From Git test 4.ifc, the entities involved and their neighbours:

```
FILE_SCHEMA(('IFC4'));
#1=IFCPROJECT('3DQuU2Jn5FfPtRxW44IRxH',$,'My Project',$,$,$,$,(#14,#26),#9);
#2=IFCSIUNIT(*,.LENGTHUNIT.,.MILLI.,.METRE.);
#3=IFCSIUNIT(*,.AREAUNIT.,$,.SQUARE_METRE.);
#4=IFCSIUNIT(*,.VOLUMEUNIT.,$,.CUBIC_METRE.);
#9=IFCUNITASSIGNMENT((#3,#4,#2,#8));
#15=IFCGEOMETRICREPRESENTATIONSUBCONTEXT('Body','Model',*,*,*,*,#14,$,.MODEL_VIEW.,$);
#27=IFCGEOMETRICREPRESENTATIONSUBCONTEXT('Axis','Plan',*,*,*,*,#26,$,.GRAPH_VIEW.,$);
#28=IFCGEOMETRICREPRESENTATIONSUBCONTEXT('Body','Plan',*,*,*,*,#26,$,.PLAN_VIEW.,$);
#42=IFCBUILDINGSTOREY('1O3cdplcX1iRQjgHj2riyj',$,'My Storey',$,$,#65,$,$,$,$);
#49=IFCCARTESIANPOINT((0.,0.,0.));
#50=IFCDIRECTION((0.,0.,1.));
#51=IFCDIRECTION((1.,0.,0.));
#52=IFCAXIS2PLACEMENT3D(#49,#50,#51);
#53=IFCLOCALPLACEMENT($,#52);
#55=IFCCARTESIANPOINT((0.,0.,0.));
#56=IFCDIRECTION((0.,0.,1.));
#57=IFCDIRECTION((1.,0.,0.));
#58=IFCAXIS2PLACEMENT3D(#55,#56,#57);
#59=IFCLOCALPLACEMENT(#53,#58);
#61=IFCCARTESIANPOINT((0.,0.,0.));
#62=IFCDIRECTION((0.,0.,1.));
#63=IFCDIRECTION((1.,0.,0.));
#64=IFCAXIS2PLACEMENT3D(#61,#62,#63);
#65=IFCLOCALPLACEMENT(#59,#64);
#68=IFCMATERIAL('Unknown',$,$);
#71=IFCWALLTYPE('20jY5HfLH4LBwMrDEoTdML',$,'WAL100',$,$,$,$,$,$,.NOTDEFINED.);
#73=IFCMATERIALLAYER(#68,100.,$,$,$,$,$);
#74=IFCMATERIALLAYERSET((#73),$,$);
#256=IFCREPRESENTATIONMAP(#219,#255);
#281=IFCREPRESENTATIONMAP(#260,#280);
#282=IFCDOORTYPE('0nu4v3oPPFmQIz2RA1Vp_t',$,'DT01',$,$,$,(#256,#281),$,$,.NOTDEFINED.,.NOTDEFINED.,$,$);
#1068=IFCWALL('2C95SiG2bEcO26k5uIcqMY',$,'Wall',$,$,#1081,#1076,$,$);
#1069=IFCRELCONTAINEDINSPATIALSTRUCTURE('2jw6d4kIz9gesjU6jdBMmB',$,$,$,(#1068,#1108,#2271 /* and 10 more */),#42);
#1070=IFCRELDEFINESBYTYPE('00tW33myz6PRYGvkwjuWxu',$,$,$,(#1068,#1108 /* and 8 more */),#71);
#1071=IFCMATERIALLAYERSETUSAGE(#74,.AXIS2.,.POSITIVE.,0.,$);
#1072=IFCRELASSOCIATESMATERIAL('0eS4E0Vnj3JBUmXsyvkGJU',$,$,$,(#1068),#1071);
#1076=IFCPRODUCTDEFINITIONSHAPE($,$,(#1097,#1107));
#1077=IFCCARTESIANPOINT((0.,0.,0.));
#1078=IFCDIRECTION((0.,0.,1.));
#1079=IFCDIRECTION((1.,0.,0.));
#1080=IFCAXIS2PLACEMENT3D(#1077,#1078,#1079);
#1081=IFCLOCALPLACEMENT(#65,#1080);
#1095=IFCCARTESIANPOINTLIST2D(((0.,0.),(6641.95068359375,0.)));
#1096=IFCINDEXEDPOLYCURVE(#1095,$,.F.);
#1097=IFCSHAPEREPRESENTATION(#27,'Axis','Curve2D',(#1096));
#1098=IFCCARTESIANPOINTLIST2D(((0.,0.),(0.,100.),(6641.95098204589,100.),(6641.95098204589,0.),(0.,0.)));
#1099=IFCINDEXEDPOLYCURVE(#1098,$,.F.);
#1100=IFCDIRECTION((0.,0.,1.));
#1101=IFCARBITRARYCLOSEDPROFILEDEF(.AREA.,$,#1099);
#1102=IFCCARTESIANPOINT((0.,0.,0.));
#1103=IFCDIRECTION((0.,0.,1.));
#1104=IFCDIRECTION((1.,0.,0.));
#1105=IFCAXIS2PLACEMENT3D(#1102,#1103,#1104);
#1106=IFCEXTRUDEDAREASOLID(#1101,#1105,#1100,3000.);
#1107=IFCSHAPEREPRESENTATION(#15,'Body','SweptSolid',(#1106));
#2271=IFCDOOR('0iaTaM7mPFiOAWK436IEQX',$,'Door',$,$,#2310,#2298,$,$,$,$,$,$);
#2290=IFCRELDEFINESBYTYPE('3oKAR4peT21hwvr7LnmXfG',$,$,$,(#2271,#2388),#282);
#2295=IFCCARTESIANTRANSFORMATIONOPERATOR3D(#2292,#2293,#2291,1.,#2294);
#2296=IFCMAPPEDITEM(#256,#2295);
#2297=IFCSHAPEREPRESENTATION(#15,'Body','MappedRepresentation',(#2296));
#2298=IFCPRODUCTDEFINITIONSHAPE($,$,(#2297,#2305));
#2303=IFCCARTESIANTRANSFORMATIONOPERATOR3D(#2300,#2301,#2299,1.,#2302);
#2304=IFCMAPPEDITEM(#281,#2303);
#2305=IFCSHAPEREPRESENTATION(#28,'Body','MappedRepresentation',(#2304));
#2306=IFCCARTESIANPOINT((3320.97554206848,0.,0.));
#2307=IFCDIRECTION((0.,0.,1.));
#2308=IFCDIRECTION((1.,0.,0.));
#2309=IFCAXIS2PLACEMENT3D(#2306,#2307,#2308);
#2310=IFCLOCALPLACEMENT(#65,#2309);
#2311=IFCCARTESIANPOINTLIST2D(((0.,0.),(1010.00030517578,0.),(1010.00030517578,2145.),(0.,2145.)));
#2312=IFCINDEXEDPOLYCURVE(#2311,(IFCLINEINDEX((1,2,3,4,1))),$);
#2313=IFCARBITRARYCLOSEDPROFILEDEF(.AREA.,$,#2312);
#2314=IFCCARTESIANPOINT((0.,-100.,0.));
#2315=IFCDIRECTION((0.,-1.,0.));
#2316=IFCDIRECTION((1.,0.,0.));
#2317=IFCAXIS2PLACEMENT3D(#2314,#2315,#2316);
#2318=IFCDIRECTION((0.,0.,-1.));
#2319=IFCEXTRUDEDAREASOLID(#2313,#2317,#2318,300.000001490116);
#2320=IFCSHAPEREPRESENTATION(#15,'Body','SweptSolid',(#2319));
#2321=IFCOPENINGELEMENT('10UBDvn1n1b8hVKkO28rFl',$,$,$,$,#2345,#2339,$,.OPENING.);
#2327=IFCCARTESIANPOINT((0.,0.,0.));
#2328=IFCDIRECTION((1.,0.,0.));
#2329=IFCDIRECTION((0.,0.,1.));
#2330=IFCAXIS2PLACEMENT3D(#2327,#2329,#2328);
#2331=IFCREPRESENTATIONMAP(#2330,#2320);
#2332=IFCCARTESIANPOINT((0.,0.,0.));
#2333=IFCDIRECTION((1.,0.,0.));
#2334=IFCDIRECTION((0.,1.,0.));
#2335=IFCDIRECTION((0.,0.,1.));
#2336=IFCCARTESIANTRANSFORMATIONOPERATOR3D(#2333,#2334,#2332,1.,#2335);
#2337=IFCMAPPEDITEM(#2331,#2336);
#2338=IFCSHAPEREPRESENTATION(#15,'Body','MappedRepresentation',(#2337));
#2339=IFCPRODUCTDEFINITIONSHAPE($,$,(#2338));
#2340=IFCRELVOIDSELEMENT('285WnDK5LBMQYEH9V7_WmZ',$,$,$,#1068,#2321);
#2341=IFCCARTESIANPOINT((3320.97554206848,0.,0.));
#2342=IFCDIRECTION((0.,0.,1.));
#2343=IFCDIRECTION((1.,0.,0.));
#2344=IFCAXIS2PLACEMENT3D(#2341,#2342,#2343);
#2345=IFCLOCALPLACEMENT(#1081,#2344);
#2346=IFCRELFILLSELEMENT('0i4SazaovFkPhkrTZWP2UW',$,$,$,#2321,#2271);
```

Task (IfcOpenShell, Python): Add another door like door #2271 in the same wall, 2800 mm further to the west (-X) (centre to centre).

```python
import ifcopenshell
import ifcopenshell.api.feature
import ifcopenshell.api.geometry
import ifcopenshell.api.root
import ifcopenshell.geom
import ifcopenshell.util.element
import ifcopenshell.util.placement
import ifcopenshell.util.shape
import ifcopenshell.util.unit

model = ifcopenshell.open("Git test 4.ifc")
unit_scale = ifcopenshell.util.unit.calculate_unit_scale(model)
settings = ifcopenshell.geom.settings()


def volume(element):
    """Net volume in cubic metres, openings subtracted."""
    shape = ifcopenshell.geom.create_shape(settings, element)
    return ifcopenshell.util.shape.get_volume(shape.geometry)


door = model.by_guid("0iaTaM7mPFiOAWK436IEQX")
opening = door.FillsVoids[0].RelatingOpeningElement
wall = opening.VoidsElements[0].RelatingBuildingElement
before = volume(wall)
shift = ifcopenshell.util.placement.get_local_placement(wall.ObjectPlacement)[:3, 0] * -2.8 / unit_scale

# copy_class copies the void relationship, type, container and properties, but no geometry.
new_opening = ifcopenshell.api.root.copy_class(model, product=opening)
new_opening.Representation = ifcopenshell.util.element.copy_deep(
    model, opening.Representation, exclude=["IfcGeometricRepresentationContext", "IfcRepresentationMap"]
)
new_door = ifcopenshell.api.root.copy_class(model, product=door)
new_door.Representation = ifcopenshell.util.element.copy_deep(
    model, door.Representation, exclude=["IfcGeometricRepresentationContext", "IfcRepresentationMap"]
)
ifcopenshell.api.feature.add_filling(model, opening=new_opening, element=new_door)

for old, new in ((opening, new_opening), (door, new_door)):
    matrix = ifcopenshell.util.placement.get_local_placement(old.ObjectPlacement)
    matrix[:3, 3] += shift
    ifcopenshell.api.geometry.edit_object_placement(model, product=new, matrix=matrix, is_si=False)

after = volume(wall)

print(f"wall volume {before:.3f} -> {after:.3f} m3")

model.write("Git test 4_rev.ifc")
```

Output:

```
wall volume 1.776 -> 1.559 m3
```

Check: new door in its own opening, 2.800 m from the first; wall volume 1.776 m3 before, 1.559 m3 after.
